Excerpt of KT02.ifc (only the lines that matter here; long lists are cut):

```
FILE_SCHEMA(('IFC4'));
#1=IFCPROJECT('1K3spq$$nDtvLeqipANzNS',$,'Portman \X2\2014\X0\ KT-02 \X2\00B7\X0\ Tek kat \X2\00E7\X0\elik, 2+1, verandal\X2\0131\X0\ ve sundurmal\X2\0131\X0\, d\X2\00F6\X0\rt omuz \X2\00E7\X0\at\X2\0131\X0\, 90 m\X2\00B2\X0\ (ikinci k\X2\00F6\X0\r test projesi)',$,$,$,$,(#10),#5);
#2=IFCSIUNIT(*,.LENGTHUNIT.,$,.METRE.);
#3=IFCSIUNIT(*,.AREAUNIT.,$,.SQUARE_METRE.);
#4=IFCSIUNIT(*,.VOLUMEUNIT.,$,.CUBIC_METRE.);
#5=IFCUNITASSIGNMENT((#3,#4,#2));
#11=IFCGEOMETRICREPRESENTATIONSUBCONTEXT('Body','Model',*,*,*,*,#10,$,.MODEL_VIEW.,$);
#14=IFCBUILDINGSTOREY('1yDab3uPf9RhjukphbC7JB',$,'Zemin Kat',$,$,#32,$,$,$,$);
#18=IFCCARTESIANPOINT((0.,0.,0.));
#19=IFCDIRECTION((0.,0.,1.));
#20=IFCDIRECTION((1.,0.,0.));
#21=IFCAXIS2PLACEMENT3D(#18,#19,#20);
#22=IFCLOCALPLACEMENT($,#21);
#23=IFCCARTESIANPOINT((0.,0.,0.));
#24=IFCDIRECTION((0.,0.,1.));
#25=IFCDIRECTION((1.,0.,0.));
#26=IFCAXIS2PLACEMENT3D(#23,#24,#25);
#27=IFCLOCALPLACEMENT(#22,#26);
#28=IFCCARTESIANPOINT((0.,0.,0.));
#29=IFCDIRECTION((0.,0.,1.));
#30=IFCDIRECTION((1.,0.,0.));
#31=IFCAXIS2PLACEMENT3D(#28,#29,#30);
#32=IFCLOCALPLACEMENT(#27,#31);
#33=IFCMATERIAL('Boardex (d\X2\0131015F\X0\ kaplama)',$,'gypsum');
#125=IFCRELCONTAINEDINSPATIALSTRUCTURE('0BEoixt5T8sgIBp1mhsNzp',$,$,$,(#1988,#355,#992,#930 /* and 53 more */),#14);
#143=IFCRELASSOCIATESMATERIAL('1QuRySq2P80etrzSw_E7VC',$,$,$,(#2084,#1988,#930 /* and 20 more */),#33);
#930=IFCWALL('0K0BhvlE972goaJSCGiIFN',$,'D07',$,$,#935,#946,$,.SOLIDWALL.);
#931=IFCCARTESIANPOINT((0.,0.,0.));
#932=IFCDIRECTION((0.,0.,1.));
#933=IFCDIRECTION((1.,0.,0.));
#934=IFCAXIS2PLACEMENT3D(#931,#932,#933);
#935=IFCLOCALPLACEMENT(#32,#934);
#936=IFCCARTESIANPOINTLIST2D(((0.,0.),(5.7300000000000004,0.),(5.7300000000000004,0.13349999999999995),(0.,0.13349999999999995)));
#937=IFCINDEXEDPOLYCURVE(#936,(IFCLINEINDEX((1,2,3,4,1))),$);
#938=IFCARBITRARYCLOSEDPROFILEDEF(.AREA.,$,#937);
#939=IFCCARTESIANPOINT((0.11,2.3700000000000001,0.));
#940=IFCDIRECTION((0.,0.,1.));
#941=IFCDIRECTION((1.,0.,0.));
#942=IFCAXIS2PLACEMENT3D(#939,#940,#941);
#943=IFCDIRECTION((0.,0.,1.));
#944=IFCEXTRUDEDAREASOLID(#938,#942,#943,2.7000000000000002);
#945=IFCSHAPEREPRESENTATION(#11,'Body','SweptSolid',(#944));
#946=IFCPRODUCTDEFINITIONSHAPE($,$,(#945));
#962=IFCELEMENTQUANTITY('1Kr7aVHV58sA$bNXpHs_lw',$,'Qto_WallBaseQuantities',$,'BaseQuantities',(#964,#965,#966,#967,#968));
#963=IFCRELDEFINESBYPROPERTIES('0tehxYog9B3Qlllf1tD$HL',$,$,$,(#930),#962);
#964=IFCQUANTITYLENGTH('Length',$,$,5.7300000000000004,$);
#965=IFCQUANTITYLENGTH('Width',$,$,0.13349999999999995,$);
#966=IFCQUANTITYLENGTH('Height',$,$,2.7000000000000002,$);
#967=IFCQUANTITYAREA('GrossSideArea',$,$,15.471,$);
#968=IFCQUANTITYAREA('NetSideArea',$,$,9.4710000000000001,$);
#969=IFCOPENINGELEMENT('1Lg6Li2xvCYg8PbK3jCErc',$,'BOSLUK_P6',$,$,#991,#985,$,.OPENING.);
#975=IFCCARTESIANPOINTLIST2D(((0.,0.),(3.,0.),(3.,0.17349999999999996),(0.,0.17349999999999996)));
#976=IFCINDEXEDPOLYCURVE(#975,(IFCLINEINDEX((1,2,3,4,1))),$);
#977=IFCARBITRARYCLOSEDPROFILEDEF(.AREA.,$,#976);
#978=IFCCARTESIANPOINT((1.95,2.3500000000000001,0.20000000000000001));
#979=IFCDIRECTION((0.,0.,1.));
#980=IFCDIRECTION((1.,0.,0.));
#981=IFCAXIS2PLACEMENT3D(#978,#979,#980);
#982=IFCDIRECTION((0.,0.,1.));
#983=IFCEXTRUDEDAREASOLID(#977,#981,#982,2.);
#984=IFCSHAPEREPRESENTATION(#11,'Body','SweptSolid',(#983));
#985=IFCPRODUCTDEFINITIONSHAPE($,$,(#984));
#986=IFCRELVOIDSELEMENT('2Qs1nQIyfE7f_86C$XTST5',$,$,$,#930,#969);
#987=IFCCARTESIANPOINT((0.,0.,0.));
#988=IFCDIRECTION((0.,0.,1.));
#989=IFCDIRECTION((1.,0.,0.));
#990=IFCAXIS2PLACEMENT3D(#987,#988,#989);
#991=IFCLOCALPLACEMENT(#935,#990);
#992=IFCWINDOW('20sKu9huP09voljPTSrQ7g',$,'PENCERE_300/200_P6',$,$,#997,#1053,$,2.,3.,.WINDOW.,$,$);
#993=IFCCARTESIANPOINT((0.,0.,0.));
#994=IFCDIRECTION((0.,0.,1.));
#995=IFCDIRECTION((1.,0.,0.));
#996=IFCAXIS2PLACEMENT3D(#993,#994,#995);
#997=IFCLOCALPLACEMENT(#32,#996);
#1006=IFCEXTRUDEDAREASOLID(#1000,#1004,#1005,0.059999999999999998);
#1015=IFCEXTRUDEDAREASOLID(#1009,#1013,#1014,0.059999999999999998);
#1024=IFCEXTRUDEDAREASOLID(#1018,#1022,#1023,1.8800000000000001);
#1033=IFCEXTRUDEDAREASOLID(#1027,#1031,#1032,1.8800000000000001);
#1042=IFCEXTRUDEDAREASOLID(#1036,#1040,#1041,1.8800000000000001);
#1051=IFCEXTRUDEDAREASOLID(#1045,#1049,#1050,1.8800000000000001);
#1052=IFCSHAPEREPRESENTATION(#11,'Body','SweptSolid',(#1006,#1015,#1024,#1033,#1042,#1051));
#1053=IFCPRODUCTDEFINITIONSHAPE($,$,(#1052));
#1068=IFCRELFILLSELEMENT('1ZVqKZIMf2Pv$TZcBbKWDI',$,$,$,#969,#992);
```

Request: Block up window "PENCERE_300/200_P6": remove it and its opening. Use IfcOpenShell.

```python
import ifcopenshell
import ifcopenshell.api.feature
import ifcopenshell.api.pset
import ifcopenshell.api.root
import ifcopenshell.geom
import ifcopenshell.util.element
import ifcopenshell.util.shape
import ifcopenshell.util.unit

model = ifcopenshell.open("KT02.ifc")
area_scale = ifcopenshell.util.unit.calculate_unit_scale(model, "AREAUNIT")
settings = ifcopenshell.geom.settings()


def volume(element):
    """Net volume in cubic metres, openings subtracted."""
    shape = ifcopenshell.geom.create_shape(settings, element)
    return ifcopenshell.util.shape.get_volume(shape.geometry)


window = model.by_guid("20sKu9huP09voljPTSrQ7g")
opening = window.FillsVoids[0].RelatingOpeningElement
wall = opening.VoidsElements[0].RelatingBuildingElement
before = volume(wall)

ifcopenshell.api.root.remove_product(model, product=window)
ifcopenshell.api.feature.remove_feature(model, feature=opening)

after = volume(wall)
thickness = 0.1335  # wall thickness in metres

# Update the wall's stored quantities.
qto = model.by_id(ifcopenshell.util.element.get_pset(wall, "Qto_WallBaseQuantities", should_inherit=False)["id"])
ifcopenshell.api.pset.edit_qto(model, qto=qto, properties={"NetSideArea": after / thickness / area_scale})

print(f"wall volume {before:.3f} -> {after:.3f} m3")

model.write("KT02_v2.ifc")
```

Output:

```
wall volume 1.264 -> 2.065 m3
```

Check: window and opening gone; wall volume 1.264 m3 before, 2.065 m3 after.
